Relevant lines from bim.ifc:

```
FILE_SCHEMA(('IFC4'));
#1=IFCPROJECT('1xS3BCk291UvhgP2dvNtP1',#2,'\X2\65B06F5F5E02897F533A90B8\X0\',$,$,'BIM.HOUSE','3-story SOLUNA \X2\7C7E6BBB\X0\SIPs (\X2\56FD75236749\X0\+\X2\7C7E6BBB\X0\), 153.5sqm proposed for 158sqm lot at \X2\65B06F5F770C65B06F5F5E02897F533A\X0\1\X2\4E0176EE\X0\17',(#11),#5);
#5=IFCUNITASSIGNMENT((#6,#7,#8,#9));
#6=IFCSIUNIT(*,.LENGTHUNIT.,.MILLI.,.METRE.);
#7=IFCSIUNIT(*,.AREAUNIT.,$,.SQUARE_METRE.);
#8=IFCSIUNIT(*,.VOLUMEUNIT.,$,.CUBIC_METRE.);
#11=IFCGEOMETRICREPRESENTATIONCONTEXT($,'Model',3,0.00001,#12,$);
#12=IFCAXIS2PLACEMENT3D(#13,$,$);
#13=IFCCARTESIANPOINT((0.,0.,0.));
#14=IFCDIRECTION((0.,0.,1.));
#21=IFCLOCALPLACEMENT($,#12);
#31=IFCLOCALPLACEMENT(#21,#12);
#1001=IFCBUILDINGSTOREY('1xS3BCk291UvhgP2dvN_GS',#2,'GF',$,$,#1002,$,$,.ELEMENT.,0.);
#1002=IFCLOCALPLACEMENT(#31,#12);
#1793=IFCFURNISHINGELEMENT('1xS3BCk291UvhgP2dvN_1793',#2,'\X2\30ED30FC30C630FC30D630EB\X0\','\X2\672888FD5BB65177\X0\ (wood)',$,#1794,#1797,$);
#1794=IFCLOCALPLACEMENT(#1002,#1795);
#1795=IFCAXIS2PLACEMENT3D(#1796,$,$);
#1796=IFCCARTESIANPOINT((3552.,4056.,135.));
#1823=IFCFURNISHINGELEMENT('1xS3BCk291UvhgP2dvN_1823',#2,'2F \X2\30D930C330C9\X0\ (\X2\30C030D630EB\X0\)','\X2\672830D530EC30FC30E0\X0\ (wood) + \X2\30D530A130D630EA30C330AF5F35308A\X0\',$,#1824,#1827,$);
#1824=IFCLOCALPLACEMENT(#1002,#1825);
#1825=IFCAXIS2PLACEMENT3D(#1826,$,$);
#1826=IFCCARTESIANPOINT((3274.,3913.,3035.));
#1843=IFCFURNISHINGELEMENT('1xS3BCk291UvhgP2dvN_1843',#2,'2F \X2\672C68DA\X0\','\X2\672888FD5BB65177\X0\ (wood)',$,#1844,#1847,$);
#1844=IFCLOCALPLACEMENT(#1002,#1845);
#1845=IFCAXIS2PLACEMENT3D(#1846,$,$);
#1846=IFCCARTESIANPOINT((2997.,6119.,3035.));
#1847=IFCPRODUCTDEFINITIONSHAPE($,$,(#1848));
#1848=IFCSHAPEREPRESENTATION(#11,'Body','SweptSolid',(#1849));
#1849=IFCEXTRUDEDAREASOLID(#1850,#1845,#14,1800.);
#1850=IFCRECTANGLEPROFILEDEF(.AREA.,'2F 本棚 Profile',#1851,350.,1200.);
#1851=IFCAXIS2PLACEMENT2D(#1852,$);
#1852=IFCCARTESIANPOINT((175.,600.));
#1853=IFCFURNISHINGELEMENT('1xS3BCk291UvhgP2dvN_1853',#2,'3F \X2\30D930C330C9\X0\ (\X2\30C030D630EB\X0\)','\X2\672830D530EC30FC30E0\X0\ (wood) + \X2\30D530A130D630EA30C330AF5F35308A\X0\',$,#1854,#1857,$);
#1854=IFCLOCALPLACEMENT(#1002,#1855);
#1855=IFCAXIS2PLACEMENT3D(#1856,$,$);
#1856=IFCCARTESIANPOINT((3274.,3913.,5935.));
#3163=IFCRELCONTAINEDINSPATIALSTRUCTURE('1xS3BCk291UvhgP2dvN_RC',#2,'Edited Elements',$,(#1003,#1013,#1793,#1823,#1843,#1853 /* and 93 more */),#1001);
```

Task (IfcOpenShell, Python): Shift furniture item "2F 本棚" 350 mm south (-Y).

```python
import ifcopenshell
import ifcopenshell.api.geometry
import ifcopenshell.util.placement
import ifcopenshell.util.unit

model = ifcopenshell.open("bim.ifc")
unit_scale = ifcopenshell.util.unit.calculate_unit_scale(model)

item = model.by_guid("1xS3BCk291UvhgP2dvN_1843")
matrix = ifcopenshell.util.placement.get_local_placement(item.ObjectPlacement)
matrix[1, 3] -= 0.35 / unit_scale
ifcopenshell.api.geometry.edit_object_placement(model, product=item, matrix=matrix, is_si=False)

print(ifcopenshell.util.placement.get_local_placement(item.ObjectPlacement).round(3) + 0.0)

model.write("bim-out.ifc")
```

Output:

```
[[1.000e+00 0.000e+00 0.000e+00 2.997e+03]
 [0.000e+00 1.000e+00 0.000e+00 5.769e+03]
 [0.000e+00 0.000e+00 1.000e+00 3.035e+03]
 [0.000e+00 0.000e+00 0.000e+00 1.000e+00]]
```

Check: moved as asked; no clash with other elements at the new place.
